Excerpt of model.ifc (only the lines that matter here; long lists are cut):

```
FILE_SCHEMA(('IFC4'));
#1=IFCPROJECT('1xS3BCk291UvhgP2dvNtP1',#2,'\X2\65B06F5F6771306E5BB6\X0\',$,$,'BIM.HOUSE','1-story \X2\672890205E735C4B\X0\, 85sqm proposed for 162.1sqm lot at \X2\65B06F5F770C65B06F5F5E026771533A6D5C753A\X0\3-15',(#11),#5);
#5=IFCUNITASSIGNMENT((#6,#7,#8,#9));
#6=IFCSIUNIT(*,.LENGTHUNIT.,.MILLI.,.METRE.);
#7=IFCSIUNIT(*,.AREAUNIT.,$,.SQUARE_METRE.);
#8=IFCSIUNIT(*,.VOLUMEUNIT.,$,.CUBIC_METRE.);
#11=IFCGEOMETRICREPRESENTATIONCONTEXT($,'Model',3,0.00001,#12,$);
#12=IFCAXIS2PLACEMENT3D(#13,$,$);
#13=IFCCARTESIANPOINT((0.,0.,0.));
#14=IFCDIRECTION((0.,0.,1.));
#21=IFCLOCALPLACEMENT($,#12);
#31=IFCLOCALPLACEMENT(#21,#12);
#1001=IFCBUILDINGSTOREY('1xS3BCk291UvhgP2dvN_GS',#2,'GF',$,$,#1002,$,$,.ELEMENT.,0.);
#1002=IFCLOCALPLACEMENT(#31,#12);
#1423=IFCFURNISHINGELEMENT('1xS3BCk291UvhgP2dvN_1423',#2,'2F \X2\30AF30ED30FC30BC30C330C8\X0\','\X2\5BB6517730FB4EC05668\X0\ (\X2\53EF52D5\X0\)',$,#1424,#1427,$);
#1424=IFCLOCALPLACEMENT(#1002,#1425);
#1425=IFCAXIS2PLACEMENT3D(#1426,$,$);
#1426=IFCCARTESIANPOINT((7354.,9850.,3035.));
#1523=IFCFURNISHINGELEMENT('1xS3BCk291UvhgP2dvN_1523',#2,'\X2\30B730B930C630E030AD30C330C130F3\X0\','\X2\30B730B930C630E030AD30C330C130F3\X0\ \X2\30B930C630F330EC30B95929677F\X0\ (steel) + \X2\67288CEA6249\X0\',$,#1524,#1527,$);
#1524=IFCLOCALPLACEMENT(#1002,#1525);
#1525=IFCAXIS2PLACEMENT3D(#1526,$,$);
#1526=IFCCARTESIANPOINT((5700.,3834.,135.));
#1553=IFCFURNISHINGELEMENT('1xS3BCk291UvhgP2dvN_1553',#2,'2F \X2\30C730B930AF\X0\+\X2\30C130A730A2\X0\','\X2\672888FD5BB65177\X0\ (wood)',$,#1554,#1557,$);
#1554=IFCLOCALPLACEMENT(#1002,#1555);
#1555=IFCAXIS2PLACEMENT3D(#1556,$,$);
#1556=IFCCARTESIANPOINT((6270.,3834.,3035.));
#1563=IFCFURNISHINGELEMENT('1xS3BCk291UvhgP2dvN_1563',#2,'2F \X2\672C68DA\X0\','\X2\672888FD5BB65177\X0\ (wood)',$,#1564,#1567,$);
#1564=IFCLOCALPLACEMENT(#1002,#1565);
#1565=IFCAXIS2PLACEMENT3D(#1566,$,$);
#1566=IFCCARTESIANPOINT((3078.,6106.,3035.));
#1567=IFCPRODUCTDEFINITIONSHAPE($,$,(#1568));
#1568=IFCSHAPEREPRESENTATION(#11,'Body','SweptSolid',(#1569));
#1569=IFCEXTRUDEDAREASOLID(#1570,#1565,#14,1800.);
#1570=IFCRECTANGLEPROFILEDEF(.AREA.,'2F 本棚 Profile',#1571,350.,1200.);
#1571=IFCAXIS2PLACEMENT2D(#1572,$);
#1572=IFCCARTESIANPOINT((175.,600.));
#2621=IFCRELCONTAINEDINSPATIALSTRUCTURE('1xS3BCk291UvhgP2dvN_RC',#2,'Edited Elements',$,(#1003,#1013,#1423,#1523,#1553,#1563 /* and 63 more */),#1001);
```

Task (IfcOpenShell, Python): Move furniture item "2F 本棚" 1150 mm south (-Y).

```python
import ifcopenshell
import ifcopenshell.api.geometry
import ifcopenshell.util.placement
import ifcopenshell.util.unit

model = ifcopenshell.open("model.ifc")
unit_scale = ifcopenshell.util.unit.calculate_unit_scale(model)

item = model.by_guid("1xS3BCk291UvhgP2dvN_1563")
matrix = ifcopenshell.util.placement.get_local_placement(item.ObjectPlacement)
matrix[1, 3] -= 1.15 / unit_scale
ifcopenshell.api.geometry.edit_object_placement(model, product=item, matrix=matrix, is_si=False)

print(ifcopenshell.util.placement.get_local_placement(item.ObjectPlacement).round(3) + 0.0)

model.write("model_v2.ifc")
```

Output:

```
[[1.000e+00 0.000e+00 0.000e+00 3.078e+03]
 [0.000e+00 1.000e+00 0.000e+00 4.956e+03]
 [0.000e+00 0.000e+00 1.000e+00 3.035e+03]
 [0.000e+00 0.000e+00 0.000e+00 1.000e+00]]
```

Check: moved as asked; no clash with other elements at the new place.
